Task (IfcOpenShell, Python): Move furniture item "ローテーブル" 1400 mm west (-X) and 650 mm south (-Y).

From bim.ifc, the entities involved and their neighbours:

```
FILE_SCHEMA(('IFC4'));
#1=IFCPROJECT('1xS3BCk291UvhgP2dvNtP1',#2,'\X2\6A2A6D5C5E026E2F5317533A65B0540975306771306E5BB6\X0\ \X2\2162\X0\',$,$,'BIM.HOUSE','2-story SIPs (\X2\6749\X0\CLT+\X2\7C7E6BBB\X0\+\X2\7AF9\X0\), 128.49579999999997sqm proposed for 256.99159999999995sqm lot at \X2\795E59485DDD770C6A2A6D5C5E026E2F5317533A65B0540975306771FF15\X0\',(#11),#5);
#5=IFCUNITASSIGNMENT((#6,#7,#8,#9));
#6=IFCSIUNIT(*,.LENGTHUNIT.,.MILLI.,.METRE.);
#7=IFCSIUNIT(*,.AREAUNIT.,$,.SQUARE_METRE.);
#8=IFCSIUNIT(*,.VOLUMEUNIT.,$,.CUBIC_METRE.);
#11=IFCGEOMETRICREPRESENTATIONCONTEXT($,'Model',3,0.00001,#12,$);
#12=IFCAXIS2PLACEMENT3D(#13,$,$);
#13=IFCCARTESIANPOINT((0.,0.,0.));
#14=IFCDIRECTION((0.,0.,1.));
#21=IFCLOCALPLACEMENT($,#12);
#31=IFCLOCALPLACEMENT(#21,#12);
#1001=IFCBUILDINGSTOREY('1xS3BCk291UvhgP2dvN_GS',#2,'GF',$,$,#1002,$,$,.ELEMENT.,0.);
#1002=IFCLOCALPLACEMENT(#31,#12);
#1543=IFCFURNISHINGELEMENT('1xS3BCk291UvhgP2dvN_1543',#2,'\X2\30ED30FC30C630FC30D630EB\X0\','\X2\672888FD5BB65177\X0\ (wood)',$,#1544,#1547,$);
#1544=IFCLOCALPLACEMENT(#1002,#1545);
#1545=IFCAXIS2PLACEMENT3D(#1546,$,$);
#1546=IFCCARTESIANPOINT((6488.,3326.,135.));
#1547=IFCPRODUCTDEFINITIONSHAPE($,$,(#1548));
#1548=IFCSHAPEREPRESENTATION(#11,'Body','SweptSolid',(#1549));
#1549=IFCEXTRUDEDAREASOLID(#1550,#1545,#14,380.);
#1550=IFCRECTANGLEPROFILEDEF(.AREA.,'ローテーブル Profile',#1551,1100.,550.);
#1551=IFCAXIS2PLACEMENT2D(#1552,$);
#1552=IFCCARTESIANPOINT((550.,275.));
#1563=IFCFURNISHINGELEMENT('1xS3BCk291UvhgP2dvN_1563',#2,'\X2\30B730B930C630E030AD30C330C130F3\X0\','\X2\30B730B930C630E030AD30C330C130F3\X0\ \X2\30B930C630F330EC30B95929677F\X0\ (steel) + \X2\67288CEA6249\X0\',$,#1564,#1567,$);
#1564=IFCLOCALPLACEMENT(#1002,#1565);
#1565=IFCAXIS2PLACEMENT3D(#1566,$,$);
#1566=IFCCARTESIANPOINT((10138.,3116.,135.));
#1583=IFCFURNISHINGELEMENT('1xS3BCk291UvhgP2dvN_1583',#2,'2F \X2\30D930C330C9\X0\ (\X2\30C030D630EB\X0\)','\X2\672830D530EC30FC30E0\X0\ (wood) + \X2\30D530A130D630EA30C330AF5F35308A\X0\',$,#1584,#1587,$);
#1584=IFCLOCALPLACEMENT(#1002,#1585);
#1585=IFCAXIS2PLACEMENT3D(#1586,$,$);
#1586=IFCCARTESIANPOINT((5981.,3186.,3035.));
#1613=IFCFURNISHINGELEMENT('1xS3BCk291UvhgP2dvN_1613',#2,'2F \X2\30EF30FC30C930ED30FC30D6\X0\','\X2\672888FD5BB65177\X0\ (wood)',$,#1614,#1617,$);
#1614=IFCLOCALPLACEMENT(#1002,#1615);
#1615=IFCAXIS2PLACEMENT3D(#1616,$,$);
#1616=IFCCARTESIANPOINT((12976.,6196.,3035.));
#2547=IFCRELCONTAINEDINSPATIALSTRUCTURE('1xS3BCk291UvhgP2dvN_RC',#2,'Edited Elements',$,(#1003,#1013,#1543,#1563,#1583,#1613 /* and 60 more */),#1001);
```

```python
import ifcopenshell
import ifcopenshell.api.geometry
import ifcopenshell.util.placement
import ifcopenshell.util.unit

model = ifcopenshell.open("bim.ifc")
unit_scale = ifcopenshell.util.unit.calculate_unit_scale(model)

item = model.by_id(1543)
matrix = ifcopenshell.util.placement.get_local_placement(item.ObjectPlacement)
matrix[0, 3] -= 1.4 / unit_scale
matrix[1, 3] -= 0.65 / unit_scale
ifcopenshell.api.geometry.edit_object_placement(model, product=item, matrix=matrix, is_si=False)

print(ifcopenshell.util.placement.get_local_placement(item.ObjectPlacement).round(3) + 0.0)

model.write("bim_updated.ifc")
```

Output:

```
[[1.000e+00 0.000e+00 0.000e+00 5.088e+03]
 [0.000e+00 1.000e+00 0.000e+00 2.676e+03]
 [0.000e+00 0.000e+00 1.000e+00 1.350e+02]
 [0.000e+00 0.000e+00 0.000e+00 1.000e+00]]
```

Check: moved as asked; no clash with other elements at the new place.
